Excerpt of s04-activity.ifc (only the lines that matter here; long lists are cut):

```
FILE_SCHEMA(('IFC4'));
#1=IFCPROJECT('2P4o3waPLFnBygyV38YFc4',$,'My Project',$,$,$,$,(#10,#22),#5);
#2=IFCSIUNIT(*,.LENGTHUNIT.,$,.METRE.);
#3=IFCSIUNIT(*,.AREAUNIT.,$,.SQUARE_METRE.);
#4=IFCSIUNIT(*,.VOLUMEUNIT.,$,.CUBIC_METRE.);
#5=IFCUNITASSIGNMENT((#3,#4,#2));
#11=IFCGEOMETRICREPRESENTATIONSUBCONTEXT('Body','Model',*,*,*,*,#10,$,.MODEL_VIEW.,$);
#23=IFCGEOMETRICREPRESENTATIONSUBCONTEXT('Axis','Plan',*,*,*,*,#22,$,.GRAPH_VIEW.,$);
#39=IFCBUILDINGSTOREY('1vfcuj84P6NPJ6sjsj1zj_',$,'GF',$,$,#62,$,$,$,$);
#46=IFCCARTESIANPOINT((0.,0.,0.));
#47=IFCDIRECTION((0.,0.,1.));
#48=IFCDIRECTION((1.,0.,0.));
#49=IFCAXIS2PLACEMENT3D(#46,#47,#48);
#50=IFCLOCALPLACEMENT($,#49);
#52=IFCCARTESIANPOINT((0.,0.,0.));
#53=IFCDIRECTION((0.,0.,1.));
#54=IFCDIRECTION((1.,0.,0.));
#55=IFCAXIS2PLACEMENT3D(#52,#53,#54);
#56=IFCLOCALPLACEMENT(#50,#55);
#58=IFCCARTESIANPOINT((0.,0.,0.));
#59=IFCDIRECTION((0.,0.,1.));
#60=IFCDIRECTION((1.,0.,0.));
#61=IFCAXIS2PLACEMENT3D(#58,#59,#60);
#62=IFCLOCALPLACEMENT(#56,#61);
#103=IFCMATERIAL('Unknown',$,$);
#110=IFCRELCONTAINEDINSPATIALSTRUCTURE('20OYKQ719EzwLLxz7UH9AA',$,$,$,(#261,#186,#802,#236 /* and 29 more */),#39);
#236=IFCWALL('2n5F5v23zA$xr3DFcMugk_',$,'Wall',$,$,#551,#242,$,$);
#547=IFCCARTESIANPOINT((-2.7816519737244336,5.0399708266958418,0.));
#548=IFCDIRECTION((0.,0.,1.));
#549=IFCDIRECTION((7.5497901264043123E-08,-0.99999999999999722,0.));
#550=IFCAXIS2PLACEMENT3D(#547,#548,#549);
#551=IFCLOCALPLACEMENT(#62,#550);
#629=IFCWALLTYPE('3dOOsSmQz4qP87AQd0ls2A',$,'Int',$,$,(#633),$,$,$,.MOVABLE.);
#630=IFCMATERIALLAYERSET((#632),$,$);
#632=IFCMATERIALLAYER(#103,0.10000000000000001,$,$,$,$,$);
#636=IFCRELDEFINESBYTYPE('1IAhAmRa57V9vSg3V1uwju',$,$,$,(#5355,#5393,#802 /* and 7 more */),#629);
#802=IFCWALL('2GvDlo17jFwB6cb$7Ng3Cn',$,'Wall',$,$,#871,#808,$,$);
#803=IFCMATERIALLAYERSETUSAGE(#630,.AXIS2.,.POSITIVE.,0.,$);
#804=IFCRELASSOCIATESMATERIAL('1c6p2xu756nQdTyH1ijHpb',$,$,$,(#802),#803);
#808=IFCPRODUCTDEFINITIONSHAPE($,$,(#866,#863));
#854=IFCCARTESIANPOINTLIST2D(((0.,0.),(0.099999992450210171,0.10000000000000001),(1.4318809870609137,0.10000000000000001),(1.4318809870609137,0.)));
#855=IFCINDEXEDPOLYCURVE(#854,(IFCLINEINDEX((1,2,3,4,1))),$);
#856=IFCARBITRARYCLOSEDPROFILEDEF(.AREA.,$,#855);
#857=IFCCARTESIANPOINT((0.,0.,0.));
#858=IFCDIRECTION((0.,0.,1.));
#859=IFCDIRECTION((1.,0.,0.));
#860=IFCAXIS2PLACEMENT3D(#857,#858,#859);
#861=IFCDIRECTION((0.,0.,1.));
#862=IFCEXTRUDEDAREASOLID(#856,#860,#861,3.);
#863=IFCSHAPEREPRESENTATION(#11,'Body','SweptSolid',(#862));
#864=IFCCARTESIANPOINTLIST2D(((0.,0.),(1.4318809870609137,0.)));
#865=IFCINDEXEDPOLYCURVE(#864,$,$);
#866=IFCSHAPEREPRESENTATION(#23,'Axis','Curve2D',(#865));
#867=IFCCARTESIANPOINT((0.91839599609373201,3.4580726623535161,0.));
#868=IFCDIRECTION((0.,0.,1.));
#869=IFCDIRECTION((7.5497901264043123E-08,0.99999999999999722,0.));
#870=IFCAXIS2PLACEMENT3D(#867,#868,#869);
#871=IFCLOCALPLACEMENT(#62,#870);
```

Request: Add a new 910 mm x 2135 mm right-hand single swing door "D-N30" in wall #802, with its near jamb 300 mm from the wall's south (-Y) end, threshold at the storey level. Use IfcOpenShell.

```python
import numpy as np
import ifcopenshell
import ifcopenshell.api.feature
import ifcopenshell.api.geometry
import ifcopenshell.api.root
import ifcopenshell.api.spatial
import ifcopenshell.geom
import ifcopenshell.util.element
import ifcopenshell.util.placement
import ifcopenshell.util.representation
import ifcopenshell.util.shape
import ifcopenshell.util.unit

model = ifcopenshell.open("s04-activity.ifc")
unit_scale = ifcopenshell.util.unit.calculate_unit_scale(model)
settings = ifcopenshell.geom.settings()


def volume(element):
    """Net volume in cubic metres, openings subtracted."""
    shape = ifcopenshell.geom.create_shape(settings, element)
    return ifcopenshell.util.shape.get_volume(shape.geometry)


wall = model.by_id(802)
storey = ifcopenshell.util.element.get_container(wall, ifc_class="IfcBuildingStorey")
context = ifcopenshell.util.representation.get_context(model, "Model", "Body", "MODEL_VIEW")
before = volume(wall)

width, height, from_end, sill = 0.91, 2.135, 0.3, 0.0  # metres

# The wall runs along its own X axis, and the end named is its -X end.
wall_shape = ifcopenshell.geom.create_shape(settings, wall)
x, y, z = ifcopenshell.util.shape.get_vertices(wall_shape.geometry).T
start = x.min() + from_end
face, thickness = float(y.min()), float(y.max() - y.min())
wall_matrix = ifcopenshell.util.placement.get_local_placement(wall.ObjectPlacement)
level = ifcopenshell.util.placement.get_local_placement(storey.ObjectPlacement)[2, 3]


def in_wall(x, y):
    """Placement at x, y metres in the wall's axes, at sill height."""
    matrix = wall_matrix.copy()
    matrix[:, 3] = wall_matrix @ np.array([x / unit_scale, y / unit_scale, 0.0, 1.0])
    matrix[2, 3] = level + sill / unit_scale
    return matrix


# Opening: a box that overshoots both wall faces by 50 mm.
opening = ifcopenshell.api.root.create_entity(model, ifc_class="IfcOpeningElement", predefined_type="OPENING")
box = ifcopenshell.api.geometry.add_wall_representation(
    model, context=context, length=width, height=height, thickness=thickness + 0.1
)
ifcopenshell.api.geometry.assign_representation(model, product=opening, representation=box)
ifcopenshell.api.geometry.edit_object_placement(model, product=opening, matrix=in_wall(start, face - 0.05), is_si=False)
ifcopenshell.api.feature.add_feature(model, feature=opening, element=wall)

door = ifcopenshell.api.root.create_entity(model, ifc_class="IfcDoor", name="D-N30", predefined_type="DOOR")
door.OverallWidth, door.OverallHeight = width / unit_scale, height / unit_scale
door.OperationType = "SINGLE_SWING_RIGHT"
body = ifcopenshell.api.geometry.add_door_representation(
    model,
    context=context,
    overall_width=door.OverallWidth,
    overall_height=door.OverallHeight,
    operation_type="SINGLE_SWING_RIGHT",
    lining_properties={"LiningDepth": thickness / unit_scale, "ThresholdDepth": thickness / unit_scale},
)
ifcopenshell.api.geometry.assign_representation(model, product=door, representation=body)
ifcopenshell.api.spatial.assign_container(model, products=[door], relating_structure=storey)
ifcopenshell.api.feature.add_filling(model, opening=opening, element=door)

# The lining spans the wall, so the door starts at the wall face.
ifcopenshell.api.geometry.edit_object_placement(model, product=door, matrix=in_wall(start, face), is_si=False)

after = volume(wall)

print(f"wall volume {before:.3f} -> {after:.3f} m3")

model.write("s04-activity_rev.ifc")
```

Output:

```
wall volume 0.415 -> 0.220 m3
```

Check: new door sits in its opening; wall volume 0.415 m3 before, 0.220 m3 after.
